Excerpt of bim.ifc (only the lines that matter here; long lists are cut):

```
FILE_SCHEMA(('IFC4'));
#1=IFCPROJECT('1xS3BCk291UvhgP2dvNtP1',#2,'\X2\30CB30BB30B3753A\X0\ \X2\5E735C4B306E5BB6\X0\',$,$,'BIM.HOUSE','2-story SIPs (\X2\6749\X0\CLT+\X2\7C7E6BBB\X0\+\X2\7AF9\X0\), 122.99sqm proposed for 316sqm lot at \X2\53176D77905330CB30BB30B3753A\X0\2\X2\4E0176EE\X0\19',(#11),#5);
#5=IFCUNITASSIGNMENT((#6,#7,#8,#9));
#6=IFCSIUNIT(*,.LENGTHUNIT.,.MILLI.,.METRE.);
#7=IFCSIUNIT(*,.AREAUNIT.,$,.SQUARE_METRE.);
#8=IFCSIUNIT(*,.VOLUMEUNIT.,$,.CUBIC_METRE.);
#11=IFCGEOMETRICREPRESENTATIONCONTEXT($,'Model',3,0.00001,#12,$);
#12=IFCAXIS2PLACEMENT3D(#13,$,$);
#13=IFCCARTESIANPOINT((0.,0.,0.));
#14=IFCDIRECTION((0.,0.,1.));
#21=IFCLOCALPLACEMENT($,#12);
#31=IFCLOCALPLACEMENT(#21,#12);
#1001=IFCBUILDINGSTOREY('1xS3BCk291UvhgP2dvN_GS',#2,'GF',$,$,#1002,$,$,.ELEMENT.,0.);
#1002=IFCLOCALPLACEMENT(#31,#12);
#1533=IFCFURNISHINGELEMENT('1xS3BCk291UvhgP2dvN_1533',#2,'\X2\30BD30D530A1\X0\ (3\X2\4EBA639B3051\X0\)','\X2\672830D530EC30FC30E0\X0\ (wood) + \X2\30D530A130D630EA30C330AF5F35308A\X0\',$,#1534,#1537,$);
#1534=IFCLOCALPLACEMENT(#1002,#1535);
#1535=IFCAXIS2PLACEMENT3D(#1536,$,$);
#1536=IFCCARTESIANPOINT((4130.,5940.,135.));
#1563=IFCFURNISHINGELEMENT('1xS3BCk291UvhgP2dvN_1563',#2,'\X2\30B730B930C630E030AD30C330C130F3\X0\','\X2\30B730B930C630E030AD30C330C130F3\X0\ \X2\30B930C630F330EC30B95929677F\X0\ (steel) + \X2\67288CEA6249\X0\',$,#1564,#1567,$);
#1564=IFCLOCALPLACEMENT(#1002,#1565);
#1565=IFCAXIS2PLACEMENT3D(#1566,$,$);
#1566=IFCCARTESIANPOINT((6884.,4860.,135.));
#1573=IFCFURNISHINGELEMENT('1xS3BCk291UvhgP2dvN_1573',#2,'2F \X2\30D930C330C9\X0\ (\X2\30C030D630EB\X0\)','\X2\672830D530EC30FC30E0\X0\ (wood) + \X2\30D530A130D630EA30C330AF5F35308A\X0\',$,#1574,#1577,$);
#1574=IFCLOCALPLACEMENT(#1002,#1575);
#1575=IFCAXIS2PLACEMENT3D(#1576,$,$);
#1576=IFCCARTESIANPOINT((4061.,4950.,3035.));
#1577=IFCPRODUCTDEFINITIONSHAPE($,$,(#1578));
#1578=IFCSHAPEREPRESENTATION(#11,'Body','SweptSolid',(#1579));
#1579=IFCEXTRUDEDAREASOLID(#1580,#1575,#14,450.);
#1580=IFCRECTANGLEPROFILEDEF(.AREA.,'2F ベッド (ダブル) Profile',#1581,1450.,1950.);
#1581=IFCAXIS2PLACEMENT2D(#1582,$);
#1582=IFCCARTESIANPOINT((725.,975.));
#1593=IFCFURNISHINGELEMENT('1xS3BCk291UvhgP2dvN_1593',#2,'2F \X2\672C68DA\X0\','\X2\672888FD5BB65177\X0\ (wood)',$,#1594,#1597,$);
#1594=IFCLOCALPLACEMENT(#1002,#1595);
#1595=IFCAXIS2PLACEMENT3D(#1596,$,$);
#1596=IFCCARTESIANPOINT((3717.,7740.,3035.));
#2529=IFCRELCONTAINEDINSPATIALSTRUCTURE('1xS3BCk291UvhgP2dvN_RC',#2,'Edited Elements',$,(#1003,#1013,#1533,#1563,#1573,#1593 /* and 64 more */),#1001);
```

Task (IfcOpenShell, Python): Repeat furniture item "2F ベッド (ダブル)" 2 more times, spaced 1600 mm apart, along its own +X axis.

```python
import ifcopenshell
import ifcopenshell.api.geometry
import ifcopenshell.api.root
import ifcopenshell.util.element
import ifcopenshell.util.placement

model = ifcopenshell.open("bim.ifc")


def reuse_history(source, copy):
    """copy_class also copies each property set's owner history, people and application; keep the originals."""
    for rel in copy.IsDefinedBy:
        if rel.is_a("IfcRelDefinesByProperties") and (history := rel.RelatingPropertyDefinition.OwnerHistory):
            rel.RelatingPropertyDefinition.OwnerHistory = source.OwnerHistory
            ifcopenshell.util.element.remove_deep2(model, history)


source = model.by_id(1573)
base = ifcopenshell.util.placement.get_local_placement(source.ObjectPlacement)
step = base[:3, 0] * 1600.0

for i in range(1, 3):
    copy = ifcopenshell.api.root.copy_class(model, product=source)
    copy.Representation = ifcopenshell.util.element.copy_deep(
        model, source.Representation, exclude=["IfcGeometricRepresentationContext", "IfcRepresentationMap"]
    )
    reuse_history(source, copy)
    matrix = base.copy()
    matrix[:3, 3] += i * step
    print("added at", matrix[:3, 3].round(3) + 0.0)
    ifcopenshell.api.geometry.edit_object_placement(model, product=copy, matrix=matrix, is_si=False)

model.write("bim_v2.ifc")
```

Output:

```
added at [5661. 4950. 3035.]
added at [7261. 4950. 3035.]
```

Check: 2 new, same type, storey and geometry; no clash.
